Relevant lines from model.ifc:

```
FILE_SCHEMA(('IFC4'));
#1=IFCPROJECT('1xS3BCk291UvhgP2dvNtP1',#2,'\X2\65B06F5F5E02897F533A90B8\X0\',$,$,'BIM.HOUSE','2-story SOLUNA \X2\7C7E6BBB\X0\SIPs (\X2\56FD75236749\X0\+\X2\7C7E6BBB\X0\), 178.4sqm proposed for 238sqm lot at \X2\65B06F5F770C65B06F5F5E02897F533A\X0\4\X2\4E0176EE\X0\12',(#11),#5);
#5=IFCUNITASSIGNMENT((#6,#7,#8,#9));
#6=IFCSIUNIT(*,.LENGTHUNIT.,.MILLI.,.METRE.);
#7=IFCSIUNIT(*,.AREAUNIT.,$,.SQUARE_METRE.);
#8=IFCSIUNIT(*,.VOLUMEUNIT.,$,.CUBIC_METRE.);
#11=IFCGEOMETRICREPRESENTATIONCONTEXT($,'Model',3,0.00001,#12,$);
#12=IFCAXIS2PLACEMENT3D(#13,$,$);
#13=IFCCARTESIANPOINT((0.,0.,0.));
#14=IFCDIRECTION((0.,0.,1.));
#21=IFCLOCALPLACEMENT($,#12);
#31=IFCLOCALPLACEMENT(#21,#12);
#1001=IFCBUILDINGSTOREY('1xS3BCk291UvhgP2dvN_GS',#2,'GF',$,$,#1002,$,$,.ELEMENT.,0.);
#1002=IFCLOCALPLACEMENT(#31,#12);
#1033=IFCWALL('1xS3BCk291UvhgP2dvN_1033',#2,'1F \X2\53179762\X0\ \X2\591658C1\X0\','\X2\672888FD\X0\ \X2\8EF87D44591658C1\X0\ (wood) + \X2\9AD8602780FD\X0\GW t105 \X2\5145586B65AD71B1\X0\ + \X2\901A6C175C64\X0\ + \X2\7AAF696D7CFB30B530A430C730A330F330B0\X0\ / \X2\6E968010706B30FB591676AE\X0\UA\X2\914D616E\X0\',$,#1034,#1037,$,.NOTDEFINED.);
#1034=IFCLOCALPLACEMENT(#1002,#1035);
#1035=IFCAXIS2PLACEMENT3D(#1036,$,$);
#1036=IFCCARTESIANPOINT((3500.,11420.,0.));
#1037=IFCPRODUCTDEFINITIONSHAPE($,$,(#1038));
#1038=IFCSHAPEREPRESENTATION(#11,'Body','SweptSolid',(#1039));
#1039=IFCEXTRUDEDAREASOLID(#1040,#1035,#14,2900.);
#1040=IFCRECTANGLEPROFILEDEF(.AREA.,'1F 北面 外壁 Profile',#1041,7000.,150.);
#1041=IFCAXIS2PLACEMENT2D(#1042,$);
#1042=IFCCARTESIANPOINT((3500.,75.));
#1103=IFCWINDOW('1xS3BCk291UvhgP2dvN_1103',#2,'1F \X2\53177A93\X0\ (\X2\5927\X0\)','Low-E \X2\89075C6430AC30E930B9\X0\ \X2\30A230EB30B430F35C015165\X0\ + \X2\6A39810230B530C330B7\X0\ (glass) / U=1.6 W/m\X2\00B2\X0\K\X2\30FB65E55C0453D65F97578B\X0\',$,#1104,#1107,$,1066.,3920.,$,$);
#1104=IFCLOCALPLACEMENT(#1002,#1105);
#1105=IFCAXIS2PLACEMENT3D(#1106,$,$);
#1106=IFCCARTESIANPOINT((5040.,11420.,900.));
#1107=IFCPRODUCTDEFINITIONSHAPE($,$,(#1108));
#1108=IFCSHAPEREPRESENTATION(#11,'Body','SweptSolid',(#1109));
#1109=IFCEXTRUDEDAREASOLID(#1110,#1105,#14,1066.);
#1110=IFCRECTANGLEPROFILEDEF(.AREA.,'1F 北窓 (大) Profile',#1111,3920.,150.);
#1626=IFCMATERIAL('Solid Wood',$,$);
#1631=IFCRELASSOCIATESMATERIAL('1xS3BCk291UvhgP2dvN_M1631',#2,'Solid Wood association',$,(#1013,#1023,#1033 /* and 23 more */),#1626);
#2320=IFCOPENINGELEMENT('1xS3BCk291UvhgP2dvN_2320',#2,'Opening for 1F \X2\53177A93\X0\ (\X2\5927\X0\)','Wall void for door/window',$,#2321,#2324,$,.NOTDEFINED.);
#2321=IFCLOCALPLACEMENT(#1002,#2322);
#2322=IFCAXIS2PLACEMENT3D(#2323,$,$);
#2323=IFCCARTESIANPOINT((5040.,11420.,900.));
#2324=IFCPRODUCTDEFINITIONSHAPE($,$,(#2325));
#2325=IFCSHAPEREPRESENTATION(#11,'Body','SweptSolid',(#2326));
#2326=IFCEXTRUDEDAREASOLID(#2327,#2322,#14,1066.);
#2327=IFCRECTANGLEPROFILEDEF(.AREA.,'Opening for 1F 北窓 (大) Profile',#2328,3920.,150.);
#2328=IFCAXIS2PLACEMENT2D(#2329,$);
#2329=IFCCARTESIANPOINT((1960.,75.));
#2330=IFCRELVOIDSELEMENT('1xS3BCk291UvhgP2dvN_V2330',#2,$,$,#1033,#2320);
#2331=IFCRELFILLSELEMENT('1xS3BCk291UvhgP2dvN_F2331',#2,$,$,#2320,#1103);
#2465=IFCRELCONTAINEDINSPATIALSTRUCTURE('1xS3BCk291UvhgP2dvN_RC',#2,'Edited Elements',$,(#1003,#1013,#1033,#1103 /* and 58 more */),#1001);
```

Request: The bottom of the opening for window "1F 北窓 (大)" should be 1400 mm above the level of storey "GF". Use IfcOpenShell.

```python
import numpy as np
import ifcopenshell
import ifcopenshell.api.geometry
import ifcopenshell.geom
import ifcopenshell.util.element
import ifcopenshell.util.placement
import ifcopenshell.util.shape
import ifcopenshell.util.unit

model = ifcopenshell.open("model.ifc")
unit_scale = ifcopenshell.util.unit.calculate_unit_scale(model)

window = model.by_id(1103)
opening = window.FillsVoids[0].RelatingOpeningElement
storey = ifcopenshell.util.element.get_container(window, ifc_class="IfcBuildingStorey")
level = ifcopenshell.util.placement.get_local_placement(storey.ObjectPlacement)[2, 3]

# The opening's origin need not be at the sill, so measure its lowest point.
shape = ifcopenshell.geom.create_shape(ifcopenshell.geom.settings(), opening)
bottom = ifcopenshell.util.shape.get_shape_bottom_elevation(shape, shape.geometry) / unit_scale
dz = level + 1.4 / unit_scale - bottom

shift = np.array([0.0, 0.0, dz])
# The window is not placed relative to its opening, so move both.
for product in (opening, window):
    matrix = ifcopenshell.util.placement.get_local_placement(product.ObjectPlacement)
    matrix[:3, 3] += shift
    ifcopenshell.api.geometry.edit_object_placement(model, product=product, matrix=matrix, is_si=False)

print(f"moved by {dz * unit_scale:+.3f} m")

model.write("model_v2.ifc")
```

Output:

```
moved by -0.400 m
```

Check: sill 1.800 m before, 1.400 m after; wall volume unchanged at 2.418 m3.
